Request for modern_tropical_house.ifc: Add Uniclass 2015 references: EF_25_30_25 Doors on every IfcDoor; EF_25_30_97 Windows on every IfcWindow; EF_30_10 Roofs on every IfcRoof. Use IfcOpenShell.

First a look at what the model holds.

```python
import ifcopenshell

model = ifcopenshell.open("modern_tropical_house.ifc")
print(model.schema)
print("classifications:", [c.Name for c in model.by_type("IfcClassification")])
for ifc_class in ("IfcDoor", "IfcRoof", "IfcStair", "IfcWall", "IfcWindow"):
    print(ifc_class, len(model.by_type(ifc_class)))
```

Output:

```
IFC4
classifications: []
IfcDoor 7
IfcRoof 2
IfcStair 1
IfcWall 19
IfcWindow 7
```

```python
import ifcopenshell
import ifcopenshell.api.classification

model = ifcopenshell.open("modern_tropical_house.ifc")

system = ifcopenshell.api.classification.add_classification(model, classification="Uniclass 2015")

codes = {
    "IfcDoor": ("EF_25_30_25", "Doors"),
    "IfcWindow": ("EF_25_30_97", "Windows"),
    "IfcRoof": ("EF_30_10", "Roofs"),
}
for ifc_class, (code, name) in codes.items():
    products = model.by_type(ifc_class)
    ifcopenshell.api.classification.add_reference(
        model, products=products, classification=system, identification=code, name=name
    )
    print(code, len(products))

model.write("modern_tropical_house_updated.ifc")
```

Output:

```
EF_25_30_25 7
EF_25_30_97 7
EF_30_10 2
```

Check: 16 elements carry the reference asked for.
